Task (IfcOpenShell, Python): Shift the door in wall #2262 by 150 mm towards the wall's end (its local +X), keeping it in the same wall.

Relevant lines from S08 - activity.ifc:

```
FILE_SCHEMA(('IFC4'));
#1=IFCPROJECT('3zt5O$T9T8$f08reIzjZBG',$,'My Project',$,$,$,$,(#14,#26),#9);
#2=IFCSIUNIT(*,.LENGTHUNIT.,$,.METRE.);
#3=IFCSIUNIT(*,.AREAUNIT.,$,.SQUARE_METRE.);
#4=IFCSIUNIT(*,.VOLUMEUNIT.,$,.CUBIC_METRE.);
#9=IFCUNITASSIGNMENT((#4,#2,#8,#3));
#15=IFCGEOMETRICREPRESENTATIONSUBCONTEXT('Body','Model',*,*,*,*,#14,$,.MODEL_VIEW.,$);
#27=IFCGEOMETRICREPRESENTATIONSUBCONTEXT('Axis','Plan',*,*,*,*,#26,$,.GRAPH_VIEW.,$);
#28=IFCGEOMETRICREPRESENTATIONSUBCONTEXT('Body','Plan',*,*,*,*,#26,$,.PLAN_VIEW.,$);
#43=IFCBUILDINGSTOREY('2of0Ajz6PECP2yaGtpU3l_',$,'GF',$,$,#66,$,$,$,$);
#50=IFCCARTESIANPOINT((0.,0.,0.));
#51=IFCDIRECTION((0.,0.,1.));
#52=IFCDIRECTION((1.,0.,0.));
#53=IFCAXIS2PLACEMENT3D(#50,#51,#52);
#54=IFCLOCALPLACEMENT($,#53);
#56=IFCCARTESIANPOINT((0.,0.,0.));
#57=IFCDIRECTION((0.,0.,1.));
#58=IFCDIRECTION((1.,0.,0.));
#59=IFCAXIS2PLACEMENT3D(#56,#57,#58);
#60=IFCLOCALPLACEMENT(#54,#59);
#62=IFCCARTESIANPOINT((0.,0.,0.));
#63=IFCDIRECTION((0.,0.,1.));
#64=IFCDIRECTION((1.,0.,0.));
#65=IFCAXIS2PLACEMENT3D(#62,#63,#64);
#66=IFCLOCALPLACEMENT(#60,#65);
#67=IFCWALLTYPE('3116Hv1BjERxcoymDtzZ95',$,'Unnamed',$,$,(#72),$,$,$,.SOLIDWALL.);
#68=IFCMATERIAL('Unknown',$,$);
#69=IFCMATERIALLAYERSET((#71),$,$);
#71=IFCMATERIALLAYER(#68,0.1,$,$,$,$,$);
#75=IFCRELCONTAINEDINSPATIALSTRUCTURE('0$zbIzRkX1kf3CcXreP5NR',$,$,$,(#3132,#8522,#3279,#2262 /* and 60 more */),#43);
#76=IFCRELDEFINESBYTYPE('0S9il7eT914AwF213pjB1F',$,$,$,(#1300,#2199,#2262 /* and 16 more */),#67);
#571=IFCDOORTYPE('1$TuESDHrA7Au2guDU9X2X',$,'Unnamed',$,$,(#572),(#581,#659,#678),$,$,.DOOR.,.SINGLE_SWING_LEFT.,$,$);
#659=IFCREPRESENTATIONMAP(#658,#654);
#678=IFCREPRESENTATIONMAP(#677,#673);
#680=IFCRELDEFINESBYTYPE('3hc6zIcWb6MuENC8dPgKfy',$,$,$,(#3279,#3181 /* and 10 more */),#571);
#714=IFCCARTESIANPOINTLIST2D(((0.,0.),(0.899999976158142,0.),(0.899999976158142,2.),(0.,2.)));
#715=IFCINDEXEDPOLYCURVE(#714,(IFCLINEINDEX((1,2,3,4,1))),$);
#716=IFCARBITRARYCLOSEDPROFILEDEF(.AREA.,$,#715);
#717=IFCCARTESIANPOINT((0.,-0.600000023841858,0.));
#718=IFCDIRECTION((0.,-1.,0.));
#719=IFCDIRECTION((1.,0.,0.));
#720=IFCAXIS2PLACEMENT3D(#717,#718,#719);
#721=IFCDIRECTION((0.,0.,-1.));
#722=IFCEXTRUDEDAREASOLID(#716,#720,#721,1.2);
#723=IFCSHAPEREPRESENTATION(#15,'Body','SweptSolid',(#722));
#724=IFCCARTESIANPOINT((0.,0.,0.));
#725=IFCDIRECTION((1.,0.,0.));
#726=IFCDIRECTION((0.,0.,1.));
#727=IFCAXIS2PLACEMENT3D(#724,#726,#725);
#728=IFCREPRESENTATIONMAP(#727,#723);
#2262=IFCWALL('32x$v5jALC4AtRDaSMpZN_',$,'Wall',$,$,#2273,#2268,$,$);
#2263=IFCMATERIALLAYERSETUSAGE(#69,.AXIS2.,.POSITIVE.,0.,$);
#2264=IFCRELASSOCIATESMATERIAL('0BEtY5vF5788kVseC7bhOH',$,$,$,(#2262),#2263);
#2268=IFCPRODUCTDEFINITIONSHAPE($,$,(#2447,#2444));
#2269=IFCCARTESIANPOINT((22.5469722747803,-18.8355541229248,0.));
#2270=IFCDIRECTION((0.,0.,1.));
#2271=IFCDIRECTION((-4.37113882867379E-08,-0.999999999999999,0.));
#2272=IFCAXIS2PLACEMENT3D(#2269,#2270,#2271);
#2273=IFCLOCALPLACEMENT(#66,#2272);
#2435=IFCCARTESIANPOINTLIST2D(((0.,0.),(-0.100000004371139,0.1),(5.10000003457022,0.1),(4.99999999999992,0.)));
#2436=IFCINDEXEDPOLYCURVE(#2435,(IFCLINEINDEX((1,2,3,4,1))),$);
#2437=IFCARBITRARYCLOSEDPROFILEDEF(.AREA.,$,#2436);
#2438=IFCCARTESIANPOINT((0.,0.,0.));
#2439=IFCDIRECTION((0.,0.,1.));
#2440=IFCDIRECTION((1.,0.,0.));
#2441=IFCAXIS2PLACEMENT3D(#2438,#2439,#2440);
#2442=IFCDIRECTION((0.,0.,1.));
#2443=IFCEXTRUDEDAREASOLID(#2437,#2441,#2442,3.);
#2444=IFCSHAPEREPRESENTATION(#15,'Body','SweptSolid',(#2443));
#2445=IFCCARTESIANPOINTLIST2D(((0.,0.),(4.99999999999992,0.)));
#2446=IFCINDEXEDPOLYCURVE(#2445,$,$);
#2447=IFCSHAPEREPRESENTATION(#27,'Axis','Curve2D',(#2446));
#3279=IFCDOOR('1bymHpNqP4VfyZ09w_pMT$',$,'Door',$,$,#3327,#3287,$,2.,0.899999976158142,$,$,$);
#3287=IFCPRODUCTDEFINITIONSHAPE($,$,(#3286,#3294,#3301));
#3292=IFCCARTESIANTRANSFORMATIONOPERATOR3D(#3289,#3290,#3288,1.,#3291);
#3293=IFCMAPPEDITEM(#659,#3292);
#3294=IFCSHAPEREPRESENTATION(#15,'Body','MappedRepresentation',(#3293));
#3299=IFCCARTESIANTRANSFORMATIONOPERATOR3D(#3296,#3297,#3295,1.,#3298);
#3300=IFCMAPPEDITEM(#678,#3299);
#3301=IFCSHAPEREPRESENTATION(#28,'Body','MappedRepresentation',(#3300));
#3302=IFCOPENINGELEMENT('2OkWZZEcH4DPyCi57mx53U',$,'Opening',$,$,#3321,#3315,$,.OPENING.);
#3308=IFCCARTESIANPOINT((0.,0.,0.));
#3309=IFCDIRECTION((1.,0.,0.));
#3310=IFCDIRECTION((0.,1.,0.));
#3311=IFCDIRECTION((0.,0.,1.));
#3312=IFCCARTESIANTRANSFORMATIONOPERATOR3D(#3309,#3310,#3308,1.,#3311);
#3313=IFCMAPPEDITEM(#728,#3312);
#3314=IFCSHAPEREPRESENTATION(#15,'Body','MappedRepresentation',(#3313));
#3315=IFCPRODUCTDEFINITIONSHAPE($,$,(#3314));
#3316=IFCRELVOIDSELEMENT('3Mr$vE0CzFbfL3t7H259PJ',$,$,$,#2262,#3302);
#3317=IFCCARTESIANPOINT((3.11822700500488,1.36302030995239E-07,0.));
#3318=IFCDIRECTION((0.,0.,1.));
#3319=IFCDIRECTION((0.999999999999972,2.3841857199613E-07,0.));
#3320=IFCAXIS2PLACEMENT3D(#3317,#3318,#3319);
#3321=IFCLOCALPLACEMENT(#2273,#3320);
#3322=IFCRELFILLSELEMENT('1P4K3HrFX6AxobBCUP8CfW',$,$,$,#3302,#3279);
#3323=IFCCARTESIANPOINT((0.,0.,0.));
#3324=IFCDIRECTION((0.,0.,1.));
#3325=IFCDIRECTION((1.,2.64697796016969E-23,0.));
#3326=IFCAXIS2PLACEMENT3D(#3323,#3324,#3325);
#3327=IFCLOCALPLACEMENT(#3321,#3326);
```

```python
import ifcopenshell
import ifcopenshell.api.geometry
import ifcopenshell.util.placement

model = ifcopenshell.open("S08 - activity.ifc")

door = model.by_guid("1bymHpNqP4VfyZ09w_pMT$")
opening = door.FillsVoids[0].RelatingOpeningElement
wall = opening.VoidsElements[0].RelatingBuildingElement

wall_matrix = ifcopenshell.util.placement.get_local_placement(wall.ObjectPlacement)
shift = wall_matrix[:3, 0] * 0.15
before = ifcopenshell.util.placement.get_local_placement(door.ObjectPlacement)[:3, 3].copy()

# The door is placed relative to its opening, so it follows when the opening moves.
matrix = ifcopenshell.util.placement.get_local_placement(opening.ObjectPlacement)
matrix[:3, 3] += shift
ifcopenshell.api.geometry.edit_object_placement(
    model, product=opening, matrix=matrix, is_si=False, should_transform_children=True
)

after = ifcopenshell.util.placement.get_local_placement(door.ObjectPlacement)[:3, 3]
print("door moved by", (after - before).round(3) + 0.0)

model.write("S08 - activity-out.ifc")
```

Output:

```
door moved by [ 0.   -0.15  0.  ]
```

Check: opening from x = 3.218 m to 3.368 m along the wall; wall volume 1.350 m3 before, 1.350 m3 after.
